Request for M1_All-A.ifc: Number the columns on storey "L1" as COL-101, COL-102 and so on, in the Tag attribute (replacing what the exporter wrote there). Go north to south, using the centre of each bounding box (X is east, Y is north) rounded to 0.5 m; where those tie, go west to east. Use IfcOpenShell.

First a look at what the model holds.

```python
import ifcopenshell
import ifcopenshell.util.element
import ifcopenshell.util.placement

model = ifcopenshell.open("M1_All-A.ifc")
print(model.schema)
storey = next(s for s in model.by_type("IfcBuildingStorey") if s.Name == "L1")
columns = [e for e in ifcopenshell.util.element.get_decomposition(storey) if e.is_a("IfcColumn")]
for e in sorted(columns, key=lambda e: e.id()):
    origin = ifcopenshell.util.placement.get_local_placement(e.ObjectPlacement)[:3, 3]
    print(e.id(), e.Tag, e.Name, origin.round(2) + 0.0, sep=" | ")
```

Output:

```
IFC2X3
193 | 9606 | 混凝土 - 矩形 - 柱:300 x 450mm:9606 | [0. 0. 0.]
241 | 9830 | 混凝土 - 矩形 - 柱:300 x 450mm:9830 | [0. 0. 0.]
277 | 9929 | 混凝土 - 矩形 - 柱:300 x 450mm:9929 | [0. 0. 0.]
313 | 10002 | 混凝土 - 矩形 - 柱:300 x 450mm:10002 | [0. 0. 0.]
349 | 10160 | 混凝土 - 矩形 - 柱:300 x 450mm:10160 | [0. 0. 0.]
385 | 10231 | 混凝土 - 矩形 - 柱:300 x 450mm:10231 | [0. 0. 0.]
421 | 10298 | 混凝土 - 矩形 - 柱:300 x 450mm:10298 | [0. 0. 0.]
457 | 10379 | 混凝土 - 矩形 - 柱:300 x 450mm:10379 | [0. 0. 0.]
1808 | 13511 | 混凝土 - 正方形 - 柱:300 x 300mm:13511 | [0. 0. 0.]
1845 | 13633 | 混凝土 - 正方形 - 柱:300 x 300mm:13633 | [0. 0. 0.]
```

```python
import ifcopenshell
import ifcopenshell.geom
import ifcopenshell.util.element
import ifcopenshell.util.shape

model = ifcopenshell.open("M1_All-A.ifc")
settings = ifcopenshell.geom.settings()
settings.set("use-world-coords", True)


def centre(element):
    shape = ifcopenshell.geom.create_shape(settings, element)
    return ifcopenshell.util.shape.get_bbox_centroid(shape.geometry)


storey = next(s for s in model.by_type("IfcBuildingStorey") if s.Name == "L1")
columns = [e for e in ifcopenshell.util.element.get_decomposition(storey) if e.is_a("IfcColumn")]

# Insertion points can sit at a corner or the storey origin, so sort by the geometry (in metres).
centres = {e: centre(e) for e in columns}
columns.sort(key=lambda e: (-round(centres[e][1] / 0.5), centres[e][0]))

for i, e in enumerate(columns, start=1):
    number = f"COL-1{i:02d}"
    e.Tag = number
    print(e.id(), number)

model.write("M1_All-A_v2.ifc")
```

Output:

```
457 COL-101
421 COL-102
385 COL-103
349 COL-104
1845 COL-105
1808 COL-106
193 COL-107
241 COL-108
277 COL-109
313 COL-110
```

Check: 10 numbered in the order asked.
